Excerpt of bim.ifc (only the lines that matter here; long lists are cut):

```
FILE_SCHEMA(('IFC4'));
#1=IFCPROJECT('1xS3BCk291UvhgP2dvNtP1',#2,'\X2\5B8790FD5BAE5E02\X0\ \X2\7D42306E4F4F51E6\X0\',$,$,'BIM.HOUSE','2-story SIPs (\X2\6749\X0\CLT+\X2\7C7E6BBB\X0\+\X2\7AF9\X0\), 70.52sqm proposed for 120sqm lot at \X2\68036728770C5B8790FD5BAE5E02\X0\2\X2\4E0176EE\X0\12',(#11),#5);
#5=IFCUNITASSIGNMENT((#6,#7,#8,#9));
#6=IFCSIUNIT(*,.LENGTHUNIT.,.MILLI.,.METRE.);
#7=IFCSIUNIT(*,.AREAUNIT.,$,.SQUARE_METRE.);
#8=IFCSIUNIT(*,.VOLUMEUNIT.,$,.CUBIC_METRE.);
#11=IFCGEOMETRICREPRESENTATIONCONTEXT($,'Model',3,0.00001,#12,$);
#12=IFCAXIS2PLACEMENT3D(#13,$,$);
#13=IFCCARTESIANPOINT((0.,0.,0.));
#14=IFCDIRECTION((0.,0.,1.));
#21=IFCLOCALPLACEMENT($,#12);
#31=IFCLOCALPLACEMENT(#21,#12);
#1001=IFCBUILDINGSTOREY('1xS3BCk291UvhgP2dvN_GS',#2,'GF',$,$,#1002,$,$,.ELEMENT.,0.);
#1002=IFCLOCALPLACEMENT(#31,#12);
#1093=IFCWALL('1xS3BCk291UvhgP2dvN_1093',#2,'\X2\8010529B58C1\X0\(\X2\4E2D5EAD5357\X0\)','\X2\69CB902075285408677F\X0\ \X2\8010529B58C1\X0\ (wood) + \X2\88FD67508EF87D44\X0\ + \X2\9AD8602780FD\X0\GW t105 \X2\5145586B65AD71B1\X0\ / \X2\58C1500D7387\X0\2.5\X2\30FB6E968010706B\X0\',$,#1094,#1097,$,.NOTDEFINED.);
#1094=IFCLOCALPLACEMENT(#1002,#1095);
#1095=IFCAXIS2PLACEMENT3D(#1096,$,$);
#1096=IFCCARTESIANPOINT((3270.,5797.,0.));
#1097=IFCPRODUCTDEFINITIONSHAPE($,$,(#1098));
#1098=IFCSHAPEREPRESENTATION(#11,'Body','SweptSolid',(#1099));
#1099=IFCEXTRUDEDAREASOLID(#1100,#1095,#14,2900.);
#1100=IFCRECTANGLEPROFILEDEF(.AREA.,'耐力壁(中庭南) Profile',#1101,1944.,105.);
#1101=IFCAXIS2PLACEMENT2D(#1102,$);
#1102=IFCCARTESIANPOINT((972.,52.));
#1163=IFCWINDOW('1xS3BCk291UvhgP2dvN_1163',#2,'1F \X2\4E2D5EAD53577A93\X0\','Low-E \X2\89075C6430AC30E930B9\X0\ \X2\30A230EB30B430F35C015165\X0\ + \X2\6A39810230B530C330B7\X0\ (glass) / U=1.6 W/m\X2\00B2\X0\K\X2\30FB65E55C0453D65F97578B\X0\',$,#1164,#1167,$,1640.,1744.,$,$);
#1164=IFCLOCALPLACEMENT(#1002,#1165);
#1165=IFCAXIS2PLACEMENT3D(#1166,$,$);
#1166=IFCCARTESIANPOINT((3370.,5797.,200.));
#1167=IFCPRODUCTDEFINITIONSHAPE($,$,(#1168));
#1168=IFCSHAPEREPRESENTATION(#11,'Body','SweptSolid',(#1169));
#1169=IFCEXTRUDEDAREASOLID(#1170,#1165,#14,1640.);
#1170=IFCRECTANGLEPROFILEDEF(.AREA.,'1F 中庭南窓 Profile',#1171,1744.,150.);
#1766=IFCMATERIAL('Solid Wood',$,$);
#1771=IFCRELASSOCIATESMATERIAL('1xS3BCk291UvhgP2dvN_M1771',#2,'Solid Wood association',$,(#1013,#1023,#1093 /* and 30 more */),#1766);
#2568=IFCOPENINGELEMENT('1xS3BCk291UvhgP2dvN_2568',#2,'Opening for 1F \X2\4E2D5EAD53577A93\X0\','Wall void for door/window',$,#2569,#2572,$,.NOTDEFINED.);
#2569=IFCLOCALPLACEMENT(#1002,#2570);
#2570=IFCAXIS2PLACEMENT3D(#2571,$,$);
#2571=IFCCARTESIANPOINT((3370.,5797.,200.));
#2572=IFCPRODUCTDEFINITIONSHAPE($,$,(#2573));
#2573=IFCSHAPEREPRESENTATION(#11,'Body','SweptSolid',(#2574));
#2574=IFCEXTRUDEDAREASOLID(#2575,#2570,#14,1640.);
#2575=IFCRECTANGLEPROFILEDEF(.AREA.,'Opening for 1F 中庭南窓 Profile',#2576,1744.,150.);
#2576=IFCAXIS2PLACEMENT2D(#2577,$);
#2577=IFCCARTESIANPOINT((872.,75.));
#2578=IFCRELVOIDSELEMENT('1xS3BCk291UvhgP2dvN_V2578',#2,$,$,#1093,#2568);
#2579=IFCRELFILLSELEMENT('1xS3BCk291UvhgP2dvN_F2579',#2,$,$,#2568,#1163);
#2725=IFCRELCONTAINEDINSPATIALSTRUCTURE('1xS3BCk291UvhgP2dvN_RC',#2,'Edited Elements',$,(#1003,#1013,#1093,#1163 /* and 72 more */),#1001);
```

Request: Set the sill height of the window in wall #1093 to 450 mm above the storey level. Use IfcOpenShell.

```python
import numpy as np
import ifcopenshell
import ifcopenshell.api.geometry
import ifcopenshell.geom
import ifcopenshell.util.element
import ifcopenshell.util.placement
import ifcopenshell.util.shape
import ifcopenshell.util.unit

model = ifcopenshell.open("bim.ifc")
unit_scale = ifcopenshell.util.unit.calculate_unit_scale(model)

window = model.by_guid("1xS3BCk291UvhgP2dvN_1163")
opening = window.FillsVoids[0].RelatingOpeningElement
storey = ifcopenshell.util.element.get_container(window, ifc_class="IfcBuildingStorey")
level = ifcopenshell.util.placement.get_local_placement(storey.ObjectPlacement)[2, 3]

# The opening's origin need not be at the sill, so measure its lowest point.
shape = ifcopenshell.geom.create_shape(ifcopenshell.geom.settings(), opening)
bottom = ifcopenshell.util.shape.get_shape_bottom_elevation(shape, shape.geometry) / unit_scale
dz = level + 0.45 / unit_scale - bottom

shift = np.array([0.0, 0.0, dz])
# The window is not placed relative to its opening, so move both.
for product in (opening, window):
    matrix = ifcopenshell.util.placement.get_local_placement(product.ObjectPlacement)
    matrix[:3, 3] += shift
    ifcopenshell.api.geometry.edit_object_placement(model, product=product, matrix=matrix, is_si=False)

print(f"moved by {dz * unit_scale:+.3f} m")

model.write("bim_rev.ifc")
```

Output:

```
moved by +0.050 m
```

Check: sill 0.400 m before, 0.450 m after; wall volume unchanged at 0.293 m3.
